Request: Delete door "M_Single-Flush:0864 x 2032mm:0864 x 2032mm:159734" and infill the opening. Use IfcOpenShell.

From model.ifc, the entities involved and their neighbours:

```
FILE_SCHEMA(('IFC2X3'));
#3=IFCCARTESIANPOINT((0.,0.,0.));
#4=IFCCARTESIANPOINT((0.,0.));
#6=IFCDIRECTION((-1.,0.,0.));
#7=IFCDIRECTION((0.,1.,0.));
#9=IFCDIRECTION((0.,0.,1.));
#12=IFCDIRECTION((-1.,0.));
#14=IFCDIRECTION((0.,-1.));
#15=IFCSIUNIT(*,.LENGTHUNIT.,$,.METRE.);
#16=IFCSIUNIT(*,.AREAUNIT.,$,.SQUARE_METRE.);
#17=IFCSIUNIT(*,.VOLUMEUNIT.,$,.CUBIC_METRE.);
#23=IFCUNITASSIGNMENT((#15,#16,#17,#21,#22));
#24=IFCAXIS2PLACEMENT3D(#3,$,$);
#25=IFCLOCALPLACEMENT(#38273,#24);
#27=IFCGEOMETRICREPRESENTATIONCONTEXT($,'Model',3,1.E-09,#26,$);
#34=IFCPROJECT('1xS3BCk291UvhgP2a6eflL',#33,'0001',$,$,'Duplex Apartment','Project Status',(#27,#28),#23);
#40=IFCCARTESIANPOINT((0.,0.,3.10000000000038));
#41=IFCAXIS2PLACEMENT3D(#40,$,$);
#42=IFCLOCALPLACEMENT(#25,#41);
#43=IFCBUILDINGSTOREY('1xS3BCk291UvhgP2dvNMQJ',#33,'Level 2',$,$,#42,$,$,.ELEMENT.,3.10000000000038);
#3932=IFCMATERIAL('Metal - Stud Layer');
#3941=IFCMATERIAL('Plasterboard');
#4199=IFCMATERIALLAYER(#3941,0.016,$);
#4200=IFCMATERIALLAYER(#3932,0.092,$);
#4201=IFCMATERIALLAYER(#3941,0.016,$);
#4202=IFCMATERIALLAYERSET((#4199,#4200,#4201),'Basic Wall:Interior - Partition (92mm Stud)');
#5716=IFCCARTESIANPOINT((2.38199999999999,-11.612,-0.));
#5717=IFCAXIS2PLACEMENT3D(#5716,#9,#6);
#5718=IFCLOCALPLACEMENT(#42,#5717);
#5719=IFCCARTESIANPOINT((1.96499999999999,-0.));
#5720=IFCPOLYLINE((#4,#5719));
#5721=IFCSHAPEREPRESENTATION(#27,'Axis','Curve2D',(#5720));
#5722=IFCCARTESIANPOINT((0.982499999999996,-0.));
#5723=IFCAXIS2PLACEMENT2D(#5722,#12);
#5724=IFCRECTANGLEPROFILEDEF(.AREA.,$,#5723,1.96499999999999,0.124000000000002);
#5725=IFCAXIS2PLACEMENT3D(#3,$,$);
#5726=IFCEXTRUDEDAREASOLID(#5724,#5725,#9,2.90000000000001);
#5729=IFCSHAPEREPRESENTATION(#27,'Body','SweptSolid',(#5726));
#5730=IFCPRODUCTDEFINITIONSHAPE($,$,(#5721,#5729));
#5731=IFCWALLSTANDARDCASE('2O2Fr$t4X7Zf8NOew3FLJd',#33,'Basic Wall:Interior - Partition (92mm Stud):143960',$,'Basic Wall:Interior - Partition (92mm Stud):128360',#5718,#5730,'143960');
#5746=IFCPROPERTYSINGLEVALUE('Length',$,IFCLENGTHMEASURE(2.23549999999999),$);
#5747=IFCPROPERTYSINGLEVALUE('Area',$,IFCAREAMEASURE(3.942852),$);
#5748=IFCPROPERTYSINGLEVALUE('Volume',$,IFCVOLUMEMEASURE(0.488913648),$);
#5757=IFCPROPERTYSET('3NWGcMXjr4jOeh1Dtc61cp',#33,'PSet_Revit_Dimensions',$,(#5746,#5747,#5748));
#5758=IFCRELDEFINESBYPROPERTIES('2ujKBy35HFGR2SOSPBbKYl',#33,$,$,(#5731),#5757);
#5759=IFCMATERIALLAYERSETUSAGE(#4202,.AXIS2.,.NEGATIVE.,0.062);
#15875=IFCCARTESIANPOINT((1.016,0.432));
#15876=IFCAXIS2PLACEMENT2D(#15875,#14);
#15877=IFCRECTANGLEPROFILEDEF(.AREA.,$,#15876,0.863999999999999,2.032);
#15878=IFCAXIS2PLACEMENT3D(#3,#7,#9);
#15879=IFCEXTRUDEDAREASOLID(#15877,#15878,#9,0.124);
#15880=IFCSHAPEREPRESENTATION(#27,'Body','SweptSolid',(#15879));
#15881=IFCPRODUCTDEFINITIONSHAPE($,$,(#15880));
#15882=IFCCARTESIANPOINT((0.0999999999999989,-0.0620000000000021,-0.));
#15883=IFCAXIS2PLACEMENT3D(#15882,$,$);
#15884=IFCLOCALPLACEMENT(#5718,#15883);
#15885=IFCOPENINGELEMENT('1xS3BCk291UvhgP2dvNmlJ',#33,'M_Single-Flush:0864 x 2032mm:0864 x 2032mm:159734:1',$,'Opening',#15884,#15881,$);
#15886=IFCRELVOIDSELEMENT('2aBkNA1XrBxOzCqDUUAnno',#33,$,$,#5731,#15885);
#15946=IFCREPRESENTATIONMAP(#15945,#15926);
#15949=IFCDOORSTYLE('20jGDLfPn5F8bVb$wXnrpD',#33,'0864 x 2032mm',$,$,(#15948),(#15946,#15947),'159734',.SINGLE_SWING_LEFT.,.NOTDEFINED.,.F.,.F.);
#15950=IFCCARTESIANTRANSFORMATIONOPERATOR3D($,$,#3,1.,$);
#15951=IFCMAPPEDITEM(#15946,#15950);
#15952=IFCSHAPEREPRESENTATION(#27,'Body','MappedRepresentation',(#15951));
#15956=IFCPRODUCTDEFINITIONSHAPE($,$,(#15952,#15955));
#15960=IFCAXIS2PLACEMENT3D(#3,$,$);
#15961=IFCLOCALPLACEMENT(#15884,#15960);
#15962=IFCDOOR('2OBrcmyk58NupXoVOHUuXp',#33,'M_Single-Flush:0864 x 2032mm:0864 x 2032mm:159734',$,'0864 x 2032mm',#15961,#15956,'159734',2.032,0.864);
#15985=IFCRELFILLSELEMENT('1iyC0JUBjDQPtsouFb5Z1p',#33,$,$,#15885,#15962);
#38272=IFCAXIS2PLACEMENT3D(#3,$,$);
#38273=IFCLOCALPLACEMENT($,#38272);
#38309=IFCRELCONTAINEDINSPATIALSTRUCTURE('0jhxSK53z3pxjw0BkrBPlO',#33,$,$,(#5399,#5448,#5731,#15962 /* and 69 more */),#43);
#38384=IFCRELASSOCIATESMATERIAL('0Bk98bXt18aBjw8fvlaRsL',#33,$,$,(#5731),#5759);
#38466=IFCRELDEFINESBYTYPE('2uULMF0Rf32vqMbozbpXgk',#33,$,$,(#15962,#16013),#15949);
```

```python
import ifcopenshell
import ifcopenshell.api.feature
import ifcopenshell.api.pset
import ifcopenshell.api.root
import ifcopenshell.geom
import ifcopenshell.util.element
import ifcopenshell.util.shape
import ifcopenshell.util.unit

model = ifcopenshell.open("model.ifc")
area_scale = ifcopenshell.util.unit.calculate_unit_scale(model, "AREAUNIT")
volume_scale = ifcopenshell.util.unit.calculate_unit_scale(model, "VOLUMEUNIT")
settings = ifcopenshell.geom.settings()


def volume(element):
    """Net volume in cubic metres, openings subtracted."""
    shape = ifcopenshell.geom.create_shape(settings, element)
    return ifcopenshell.util.shape.get_volume(shape.geometry)


door = model.by_id(15962)
opening = door.FillsVoids[0].RelatingOpeningElement
wall = opening.VoidsElements[0].RelatingBuildingElement
before = volume(wall)

ifcopenshell.api.root.remove_product(model, product=door)
ifcopenshell.api.feature.remove_feature(model, feature=opening)

after = volume(wall)
thickness = 0.124  # wall thickness in metres

# Update the wall's stored quantities.
pset = model.by_id(ifcopenshell.util.element.get_pset(wall, "PSet_Revit_Dimensions", should_inherit=False)["id"])
ifcopenshell.api.pset.edit_pset(model, pset=pset, properties={
    "Area": model.create_entity("IfcAreaMeasure", after / thickness / area_scale),
    "Volume": model.create_entity("IfcVolumeMeasure", after / volume_scale),
})

print(f"wall volume {before:.3f} -> {after:.3f} m3")

model.write("model-out.ifc")
```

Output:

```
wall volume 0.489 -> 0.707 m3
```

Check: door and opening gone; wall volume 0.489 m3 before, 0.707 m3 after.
